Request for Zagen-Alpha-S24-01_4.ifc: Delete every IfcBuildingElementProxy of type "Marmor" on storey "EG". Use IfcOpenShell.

First a look at what the model holds.

```python
import ifcopenshell
import ifcopenshell.util.element

model = ifcopenshell.open("Zagen-Alpha-S24-01_4.ifc")
print(model.schema)
storey = next(s for s in model.by_type("IfcBuildingStorey") if s.Name == "EG")
proxies = [e for e in ifcopenshell.util.element.get_decomposition(storey) if e.is_a("IfcBuildingElementProxy")]
seen = {}
for e in proxies:
    element_type = ifcopenshell.util.element.get_type(e)
    name = element_type.Name if element_type not in (None, e) else None
    seen[name] = seen.get(name, 0) + 1
for name, count in sorted(seen.items(), key=str):
    print(count, "x", name)
```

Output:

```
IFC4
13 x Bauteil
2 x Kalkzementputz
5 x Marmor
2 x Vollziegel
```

```python
import ifcopenshell
import ifcopenshell.api.root
import ifcopenshell.util.element

model = ifcopenshell.open("Zagen-Alpha-S24-01_4.ifc")

storey = next(s for s in model.by_type("IfcBuildingStorey") if s.Name == "EG")
proxies = [e for e in ifcopenshell.util.element.get_decomposition(storey) if e.is_a("IfcBuildingElementProxy")]
targets = [e for e in proxies if (t := ifcopenshell.util.element.get_type(e)) not in (None, e) and t.Name == "Marmor"]

for e in targets:
    ifcopenshell.api.root.remove_product(model, product=e)
print(len(targets), "removed")

model.write("Zagen-Alpha-S24-01_4-out.ifc")
```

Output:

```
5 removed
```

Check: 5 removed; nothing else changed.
